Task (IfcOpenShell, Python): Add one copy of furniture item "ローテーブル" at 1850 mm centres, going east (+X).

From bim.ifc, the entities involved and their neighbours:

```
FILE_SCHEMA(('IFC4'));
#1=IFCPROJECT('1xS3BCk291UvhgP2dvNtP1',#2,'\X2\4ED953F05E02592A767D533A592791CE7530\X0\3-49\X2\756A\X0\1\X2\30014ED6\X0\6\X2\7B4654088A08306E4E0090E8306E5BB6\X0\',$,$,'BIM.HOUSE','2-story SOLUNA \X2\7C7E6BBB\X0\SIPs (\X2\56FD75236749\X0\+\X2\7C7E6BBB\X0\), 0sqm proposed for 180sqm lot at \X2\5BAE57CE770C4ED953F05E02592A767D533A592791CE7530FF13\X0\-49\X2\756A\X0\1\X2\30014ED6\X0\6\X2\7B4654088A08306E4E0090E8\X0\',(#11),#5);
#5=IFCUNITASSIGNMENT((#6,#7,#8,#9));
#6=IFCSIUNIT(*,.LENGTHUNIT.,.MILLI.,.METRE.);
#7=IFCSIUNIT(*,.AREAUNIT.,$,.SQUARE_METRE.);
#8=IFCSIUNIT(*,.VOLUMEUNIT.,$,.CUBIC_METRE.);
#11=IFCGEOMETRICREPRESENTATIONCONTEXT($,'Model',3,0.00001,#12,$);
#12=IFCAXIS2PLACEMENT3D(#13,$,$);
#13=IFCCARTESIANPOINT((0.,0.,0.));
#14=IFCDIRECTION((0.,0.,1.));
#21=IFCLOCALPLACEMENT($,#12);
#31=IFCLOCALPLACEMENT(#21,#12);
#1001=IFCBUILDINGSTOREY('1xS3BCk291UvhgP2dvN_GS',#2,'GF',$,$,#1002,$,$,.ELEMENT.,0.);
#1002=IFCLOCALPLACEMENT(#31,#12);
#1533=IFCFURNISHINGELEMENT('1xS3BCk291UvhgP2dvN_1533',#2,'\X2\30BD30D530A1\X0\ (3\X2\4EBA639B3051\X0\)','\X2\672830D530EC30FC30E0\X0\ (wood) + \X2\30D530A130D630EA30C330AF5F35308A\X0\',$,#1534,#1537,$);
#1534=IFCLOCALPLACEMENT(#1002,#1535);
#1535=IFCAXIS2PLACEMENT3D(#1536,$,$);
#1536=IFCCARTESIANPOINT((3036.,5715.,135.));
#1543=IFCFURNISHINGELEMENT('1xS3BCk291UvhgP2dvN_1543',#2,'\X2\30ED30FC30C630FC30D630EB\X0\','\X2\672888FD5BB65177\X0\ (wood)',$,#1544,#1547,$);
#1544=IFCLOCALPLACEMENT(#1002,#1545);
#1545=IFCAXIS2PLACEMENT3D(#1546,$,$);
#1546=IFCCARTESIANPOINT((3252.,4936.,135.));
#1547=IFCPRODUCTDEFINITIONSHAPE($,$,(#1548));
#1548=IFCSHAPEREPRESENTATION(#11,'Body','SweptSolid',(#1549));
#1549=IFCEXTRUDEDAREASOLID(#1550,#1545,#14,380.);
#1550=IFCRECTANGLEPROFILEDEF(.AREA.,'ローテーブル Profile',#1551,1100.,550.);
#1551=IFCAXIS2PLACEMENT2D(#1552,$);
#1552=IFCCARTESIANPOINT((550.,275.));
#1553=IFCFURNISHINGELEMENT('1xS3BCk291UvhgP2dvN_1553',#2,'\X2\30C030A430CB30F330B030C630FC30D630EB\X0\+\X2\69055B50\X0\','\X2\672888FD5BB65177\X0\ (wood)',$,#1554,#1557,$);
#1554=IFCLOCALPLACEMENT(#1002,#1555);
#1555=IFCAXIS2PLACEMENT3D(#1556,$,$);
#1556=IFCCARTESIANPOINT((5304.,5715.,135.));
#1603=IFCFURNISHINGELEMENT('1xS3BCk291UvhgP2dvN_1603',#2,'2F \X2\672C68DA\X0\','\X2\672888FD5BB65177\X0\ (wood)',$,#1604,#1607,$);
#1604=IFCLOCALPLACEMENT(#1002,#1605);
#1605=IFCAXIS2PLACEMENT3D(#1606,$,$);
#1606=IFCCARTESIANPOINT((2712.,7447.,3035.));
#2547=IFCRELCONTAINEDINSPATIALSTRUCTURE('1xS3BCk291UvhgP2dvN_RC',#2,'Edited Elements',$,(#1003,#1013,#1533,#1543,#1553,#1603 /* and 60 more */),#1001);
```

```python
import numpy as np
import ifcopenshell
import ifcopenshell.api.geometry
import ifcopenshell.api.root
import ifcopenshell.util.element
import ifcopenshell.util.placement

model = ifcopenshell.open("bim.ifc")


def reuse_history(source, copy):
    """copy_class also copies each property set's owner history, people and application; keep the originals."""
    for rel in copy.IsDefinedBy:
        if rel.is_a("IfcRelDefinesByProperties") and (history := rel.RelatingPropertyDefinition.OwnerHistory):
            rel.RelatingPropertyDefinition.OwnerHistory = source.OwnerHistory
            ifcopenshell.util.element.remove_deep2(model, history)


source = model.by_guid("1xS3BCk291UvhgP2dvN_1543")
base = ifcopenshell.util.placement.get_local_placement(source.ObjectPlacement)
step = np.array([1.0, 0.0, 0.0]) * 1850.0

for i in range(1, 2):
    copy = ifcopenshell.api.root.copy_class(model, product=source)
    copy.Representation = ifcopenshell.util.element.copy_deep(
        model, source.Representation, exclude=["IfcGeometricRepresentationContext", "IfcRepresentationMap"]
    )
    reuse_history(source, copy)
    matrix = base.copy()
    matrix[:3, 3] += i * step
    print("added at", matrix[:3, 3].round(3) + 0.0)
    ifcopenshell.api.geometry.edit_object_placement(model, product=copy, matrix=matrix, is_si=False)

model.write("bim_v2.ifc")
```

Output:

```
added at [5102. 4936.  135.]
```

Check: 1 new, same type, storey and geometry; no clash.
